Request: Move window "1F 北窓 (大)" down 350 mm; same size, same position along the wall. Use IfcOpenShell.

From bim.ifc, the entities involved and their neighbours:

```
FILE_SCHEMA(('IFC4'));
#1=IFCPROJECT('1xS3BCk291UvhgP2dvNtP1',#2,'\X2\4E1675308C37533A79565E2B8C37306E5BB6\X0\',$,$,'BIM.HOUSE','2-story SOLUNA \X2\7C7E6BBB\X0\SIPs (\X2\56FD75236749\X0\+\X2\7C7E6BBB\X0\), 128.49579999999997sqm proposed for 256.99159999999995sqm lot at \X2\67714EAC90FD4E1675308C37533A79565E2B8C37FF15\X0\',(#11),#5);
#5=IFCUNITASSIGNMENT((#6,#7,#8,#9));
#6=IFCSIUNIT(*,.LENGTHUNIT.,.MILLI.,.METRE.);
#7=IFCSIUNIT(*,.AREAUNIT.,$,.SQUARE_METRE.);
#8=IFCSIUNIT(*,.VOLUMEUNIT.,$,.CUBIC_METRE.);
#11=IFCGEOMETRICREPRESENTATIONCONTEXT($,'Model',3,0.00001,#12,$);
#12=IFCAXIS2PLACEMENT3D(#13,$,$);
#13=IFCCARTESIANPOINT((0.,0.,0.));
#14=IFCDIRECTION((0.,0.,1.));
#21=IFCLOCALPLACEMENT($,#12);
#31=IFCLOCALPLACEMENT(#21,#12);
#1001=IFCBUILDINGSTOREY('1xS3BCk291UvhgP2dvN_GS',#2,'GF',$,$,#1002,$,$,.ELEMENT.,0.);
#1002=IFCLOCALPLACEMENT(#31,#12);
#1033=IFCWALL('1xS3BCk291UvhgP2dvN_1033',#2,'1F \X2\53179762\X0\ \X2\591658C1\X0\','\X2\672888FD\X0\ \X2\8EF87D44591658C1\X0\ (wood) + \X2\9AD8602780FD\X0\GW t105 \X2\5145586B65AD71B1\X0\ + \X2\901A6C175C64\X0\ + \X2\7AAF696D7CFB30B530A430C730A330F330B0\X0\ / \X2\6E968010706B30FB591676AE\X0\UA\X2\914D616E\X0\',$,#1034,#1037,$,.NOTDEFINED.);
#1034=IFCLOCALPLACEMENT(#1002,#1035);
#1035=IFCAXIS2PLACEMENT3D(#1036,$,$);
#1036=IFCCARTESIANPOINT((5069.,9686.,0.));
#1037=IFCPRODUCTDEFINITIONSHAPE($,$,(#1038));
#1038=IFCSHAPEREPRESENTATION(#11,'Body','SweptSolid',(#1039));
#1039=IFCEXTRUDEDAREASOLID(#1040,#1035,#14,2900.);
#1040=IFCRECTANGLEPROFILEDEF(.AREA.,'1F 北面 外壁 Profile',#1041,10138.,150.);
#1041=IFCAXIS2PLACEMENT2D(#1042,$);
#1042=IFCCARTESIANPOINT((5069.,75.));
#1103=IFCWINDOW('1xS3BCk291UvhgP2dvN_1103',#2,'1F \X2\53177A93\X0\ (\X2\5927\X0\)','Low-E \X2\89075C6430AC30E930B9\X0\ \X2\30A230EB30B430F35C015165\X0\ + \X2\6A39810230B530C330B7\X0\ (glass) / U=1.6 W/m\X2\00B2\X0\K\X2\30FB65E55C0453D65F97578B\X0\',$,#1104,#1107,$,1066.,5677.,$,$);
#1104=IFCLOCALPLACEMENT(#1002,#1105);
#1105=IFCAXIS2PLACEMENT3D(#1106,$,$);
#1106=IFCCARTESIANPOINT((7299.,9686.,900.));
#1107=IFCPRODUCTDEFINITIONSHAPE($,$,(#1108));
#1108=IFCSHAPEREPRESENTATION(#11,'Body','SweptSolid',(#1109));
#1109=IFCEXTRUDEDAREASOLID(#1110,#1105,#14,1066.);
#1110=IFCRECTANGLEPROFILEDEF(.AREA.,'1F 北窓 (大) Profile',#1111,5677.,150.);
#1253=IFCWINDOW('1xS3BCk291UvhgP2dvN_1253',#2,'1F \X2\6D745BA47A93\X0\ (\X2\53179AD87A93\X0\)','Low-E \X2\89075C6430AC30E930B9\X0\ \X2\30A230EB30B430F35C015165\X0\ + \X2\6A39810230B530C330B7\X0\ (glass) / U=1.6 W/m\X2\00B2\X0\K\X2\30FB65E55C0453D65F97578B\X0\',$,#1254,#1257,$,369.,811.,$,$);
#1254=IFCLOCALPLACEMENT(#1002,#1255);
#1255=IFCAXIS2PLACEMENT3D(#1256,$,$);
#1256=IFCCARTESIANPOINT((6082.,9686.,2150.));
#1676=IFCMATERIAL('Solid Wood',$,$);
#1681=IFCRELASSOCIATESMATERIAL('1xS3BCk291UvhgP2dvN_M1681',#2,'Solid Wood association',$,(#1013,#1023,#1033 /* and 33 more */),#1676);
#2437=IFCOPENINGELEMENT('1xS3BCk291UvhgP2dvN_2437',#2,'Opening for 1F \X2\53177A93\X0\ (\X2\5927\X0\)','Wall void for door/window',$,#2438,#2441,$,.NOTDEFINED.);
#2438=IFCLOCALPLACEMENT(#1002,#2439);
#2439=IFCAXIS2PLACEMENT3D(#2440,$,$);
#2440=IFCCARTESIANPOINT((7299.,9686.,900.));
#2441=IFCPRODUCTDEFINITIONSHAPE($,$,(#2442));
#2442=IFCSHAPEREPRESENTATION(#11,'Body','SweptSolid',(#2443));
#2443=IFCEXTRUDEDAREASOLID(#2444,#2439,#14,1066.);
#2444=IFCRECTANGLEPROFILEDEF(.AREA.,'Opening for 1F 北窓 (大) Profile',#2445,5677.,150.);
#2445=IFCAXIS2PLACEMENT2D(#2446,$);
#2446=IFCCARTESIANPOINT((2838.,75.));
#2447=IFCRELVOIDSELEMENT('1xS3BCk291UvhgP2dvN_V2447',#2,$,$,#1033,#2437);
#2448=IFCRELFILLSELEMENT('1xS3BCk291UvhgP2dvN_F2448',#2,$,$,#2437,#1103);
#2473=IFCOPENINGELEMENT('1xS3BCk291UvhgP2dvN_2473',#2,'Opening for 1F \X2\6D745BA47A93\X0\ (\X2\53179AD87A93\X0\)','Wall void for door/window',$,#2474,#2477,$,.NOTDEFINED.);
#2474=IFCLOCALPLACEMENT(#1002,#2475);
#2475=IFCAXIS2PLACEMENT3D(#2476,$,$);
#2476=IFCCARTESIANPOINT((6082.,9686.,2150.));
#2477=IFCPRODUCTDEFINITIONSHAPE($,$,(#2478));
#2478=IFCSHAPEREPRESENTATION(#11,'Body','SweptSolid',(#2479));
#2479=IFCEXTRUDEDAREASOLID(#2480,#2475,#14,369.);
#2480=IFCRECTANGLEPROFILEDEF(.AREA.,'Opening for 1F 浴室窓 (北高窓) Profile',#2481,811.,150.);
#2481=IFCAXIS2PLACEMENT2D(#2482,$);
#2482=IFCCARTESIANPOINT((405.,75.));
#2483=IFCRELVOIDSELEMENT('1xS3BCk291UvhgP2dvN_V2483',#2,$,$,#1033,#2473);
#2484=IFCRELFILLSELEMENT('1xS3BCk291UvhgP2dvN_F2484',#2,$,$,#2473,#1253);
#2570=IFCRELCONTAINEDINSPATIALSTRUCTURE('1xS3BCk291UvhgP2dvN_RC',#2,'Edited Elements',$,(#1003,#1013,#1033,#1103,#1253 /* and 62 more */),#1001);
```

```python
import numpy as np
import ifcopenshell
import ifcopenshell.api.geometry
import ifcopenshell.util.placement
import ifcopenshell.util.unit

model = ifcopenshell.open("bim.ifc")
unit_scale = ifcopenshell.util.unit.calculate_unit_scale(model)

window = model.by_id(1103)
opening = window.FillsVoids[0].RelatingOpeningElement
dz = -0.35 / unit_scale

shift = np.array([0.0, 0.0, dz])
# The window is not placed relative to its opening, so move both.
for product in (opening, window):
    matrix = ifcopenshell.util.placement.get_local_placement(product.ObjectPlacement)
    matrix[:3, 3] += shift
    ifcopenshell.api.geometry.edit_object_placement(model, product=product, matrix=matrix, is_si=False)

print(f"moved by {dz * unit_scale:+.3f} m")

model.write("bim_updated.ifc")
```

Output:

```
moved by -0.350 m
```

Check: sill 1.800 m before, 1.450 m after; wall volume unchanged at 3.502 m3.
